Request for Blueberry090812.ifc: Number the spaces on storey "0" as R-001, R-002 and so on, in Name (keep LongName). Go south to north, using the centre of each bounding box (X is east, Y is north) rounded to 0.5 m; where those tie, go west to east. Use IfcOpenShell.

First a look at what the model holds.

```python
import ifcopenshell
import ifcopenshell.util.element
import ifcopenshell.util.placement

model = ifcopenshell.open("Blueberry090812.ifc")
print(model.schema)
storey = next(s for s in model.by_type("IfcBuildingStorey") if s.Name == "0")
spaces = [e for e in ifcopenshell.util.element.get_decomposition(storey) if e.is_a("IfcSpace")]
for e in sorted(spaces, key=lambda e: e.id()):
    origin = ifcopenshell.util.placement.get_local_placement(e.ObjectPlacement)[:3, 3]
    print(e.id(), e.Name, e.LongName, origin.round(2) + 0.0, sep=" | ")
```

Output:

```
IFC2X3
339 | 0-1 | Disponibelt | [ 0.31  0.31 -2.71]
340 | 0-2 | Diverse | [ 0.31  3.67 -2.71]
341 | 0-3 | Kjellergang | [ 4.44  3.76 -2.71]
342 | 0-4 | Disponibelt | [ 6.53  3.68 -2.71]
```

```python
import ifcopenshell
import ifcopenshell.geom
import ifcopenshell.util.element
import ifcopenshell.util.shape

model = ifcopenshell.open("Blueberry090812.ifc")
settings = ifcopenshell.geom.settings()
settings.set("use-world-coords", True)


def centre(element):
    shape = ifcopenshell.geom.create_shape(settings, element)
    return ifcopenshell.util.shape.get_bbox_centroid(shape.geometry)


storey = next(s for s in model.by_type("IfcBuildingStorey") if s.Name == "0")
spaces = [e for e in ifcopenshell.util.element.get_decomposition(storey) if e.is_a("IfcSpace")]

# Insertion points can sit at a corner or the storey origin, so sort by the geometry (in metres).
centres = {e: centre(e) for e in spaces}
spaces.sort(key=lambda e: (round(centres[e][1] / 0.5), centres[e][0]))

for i, e in enumerate(spaces, start=1):
    number = f"R-0{i:02d}"
    e.Name = number
    print(e.id(), number)

model.write("Blueberry090812-out.ifc")
```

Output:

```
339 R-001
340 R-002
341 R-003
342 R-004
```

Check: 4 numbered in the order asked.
